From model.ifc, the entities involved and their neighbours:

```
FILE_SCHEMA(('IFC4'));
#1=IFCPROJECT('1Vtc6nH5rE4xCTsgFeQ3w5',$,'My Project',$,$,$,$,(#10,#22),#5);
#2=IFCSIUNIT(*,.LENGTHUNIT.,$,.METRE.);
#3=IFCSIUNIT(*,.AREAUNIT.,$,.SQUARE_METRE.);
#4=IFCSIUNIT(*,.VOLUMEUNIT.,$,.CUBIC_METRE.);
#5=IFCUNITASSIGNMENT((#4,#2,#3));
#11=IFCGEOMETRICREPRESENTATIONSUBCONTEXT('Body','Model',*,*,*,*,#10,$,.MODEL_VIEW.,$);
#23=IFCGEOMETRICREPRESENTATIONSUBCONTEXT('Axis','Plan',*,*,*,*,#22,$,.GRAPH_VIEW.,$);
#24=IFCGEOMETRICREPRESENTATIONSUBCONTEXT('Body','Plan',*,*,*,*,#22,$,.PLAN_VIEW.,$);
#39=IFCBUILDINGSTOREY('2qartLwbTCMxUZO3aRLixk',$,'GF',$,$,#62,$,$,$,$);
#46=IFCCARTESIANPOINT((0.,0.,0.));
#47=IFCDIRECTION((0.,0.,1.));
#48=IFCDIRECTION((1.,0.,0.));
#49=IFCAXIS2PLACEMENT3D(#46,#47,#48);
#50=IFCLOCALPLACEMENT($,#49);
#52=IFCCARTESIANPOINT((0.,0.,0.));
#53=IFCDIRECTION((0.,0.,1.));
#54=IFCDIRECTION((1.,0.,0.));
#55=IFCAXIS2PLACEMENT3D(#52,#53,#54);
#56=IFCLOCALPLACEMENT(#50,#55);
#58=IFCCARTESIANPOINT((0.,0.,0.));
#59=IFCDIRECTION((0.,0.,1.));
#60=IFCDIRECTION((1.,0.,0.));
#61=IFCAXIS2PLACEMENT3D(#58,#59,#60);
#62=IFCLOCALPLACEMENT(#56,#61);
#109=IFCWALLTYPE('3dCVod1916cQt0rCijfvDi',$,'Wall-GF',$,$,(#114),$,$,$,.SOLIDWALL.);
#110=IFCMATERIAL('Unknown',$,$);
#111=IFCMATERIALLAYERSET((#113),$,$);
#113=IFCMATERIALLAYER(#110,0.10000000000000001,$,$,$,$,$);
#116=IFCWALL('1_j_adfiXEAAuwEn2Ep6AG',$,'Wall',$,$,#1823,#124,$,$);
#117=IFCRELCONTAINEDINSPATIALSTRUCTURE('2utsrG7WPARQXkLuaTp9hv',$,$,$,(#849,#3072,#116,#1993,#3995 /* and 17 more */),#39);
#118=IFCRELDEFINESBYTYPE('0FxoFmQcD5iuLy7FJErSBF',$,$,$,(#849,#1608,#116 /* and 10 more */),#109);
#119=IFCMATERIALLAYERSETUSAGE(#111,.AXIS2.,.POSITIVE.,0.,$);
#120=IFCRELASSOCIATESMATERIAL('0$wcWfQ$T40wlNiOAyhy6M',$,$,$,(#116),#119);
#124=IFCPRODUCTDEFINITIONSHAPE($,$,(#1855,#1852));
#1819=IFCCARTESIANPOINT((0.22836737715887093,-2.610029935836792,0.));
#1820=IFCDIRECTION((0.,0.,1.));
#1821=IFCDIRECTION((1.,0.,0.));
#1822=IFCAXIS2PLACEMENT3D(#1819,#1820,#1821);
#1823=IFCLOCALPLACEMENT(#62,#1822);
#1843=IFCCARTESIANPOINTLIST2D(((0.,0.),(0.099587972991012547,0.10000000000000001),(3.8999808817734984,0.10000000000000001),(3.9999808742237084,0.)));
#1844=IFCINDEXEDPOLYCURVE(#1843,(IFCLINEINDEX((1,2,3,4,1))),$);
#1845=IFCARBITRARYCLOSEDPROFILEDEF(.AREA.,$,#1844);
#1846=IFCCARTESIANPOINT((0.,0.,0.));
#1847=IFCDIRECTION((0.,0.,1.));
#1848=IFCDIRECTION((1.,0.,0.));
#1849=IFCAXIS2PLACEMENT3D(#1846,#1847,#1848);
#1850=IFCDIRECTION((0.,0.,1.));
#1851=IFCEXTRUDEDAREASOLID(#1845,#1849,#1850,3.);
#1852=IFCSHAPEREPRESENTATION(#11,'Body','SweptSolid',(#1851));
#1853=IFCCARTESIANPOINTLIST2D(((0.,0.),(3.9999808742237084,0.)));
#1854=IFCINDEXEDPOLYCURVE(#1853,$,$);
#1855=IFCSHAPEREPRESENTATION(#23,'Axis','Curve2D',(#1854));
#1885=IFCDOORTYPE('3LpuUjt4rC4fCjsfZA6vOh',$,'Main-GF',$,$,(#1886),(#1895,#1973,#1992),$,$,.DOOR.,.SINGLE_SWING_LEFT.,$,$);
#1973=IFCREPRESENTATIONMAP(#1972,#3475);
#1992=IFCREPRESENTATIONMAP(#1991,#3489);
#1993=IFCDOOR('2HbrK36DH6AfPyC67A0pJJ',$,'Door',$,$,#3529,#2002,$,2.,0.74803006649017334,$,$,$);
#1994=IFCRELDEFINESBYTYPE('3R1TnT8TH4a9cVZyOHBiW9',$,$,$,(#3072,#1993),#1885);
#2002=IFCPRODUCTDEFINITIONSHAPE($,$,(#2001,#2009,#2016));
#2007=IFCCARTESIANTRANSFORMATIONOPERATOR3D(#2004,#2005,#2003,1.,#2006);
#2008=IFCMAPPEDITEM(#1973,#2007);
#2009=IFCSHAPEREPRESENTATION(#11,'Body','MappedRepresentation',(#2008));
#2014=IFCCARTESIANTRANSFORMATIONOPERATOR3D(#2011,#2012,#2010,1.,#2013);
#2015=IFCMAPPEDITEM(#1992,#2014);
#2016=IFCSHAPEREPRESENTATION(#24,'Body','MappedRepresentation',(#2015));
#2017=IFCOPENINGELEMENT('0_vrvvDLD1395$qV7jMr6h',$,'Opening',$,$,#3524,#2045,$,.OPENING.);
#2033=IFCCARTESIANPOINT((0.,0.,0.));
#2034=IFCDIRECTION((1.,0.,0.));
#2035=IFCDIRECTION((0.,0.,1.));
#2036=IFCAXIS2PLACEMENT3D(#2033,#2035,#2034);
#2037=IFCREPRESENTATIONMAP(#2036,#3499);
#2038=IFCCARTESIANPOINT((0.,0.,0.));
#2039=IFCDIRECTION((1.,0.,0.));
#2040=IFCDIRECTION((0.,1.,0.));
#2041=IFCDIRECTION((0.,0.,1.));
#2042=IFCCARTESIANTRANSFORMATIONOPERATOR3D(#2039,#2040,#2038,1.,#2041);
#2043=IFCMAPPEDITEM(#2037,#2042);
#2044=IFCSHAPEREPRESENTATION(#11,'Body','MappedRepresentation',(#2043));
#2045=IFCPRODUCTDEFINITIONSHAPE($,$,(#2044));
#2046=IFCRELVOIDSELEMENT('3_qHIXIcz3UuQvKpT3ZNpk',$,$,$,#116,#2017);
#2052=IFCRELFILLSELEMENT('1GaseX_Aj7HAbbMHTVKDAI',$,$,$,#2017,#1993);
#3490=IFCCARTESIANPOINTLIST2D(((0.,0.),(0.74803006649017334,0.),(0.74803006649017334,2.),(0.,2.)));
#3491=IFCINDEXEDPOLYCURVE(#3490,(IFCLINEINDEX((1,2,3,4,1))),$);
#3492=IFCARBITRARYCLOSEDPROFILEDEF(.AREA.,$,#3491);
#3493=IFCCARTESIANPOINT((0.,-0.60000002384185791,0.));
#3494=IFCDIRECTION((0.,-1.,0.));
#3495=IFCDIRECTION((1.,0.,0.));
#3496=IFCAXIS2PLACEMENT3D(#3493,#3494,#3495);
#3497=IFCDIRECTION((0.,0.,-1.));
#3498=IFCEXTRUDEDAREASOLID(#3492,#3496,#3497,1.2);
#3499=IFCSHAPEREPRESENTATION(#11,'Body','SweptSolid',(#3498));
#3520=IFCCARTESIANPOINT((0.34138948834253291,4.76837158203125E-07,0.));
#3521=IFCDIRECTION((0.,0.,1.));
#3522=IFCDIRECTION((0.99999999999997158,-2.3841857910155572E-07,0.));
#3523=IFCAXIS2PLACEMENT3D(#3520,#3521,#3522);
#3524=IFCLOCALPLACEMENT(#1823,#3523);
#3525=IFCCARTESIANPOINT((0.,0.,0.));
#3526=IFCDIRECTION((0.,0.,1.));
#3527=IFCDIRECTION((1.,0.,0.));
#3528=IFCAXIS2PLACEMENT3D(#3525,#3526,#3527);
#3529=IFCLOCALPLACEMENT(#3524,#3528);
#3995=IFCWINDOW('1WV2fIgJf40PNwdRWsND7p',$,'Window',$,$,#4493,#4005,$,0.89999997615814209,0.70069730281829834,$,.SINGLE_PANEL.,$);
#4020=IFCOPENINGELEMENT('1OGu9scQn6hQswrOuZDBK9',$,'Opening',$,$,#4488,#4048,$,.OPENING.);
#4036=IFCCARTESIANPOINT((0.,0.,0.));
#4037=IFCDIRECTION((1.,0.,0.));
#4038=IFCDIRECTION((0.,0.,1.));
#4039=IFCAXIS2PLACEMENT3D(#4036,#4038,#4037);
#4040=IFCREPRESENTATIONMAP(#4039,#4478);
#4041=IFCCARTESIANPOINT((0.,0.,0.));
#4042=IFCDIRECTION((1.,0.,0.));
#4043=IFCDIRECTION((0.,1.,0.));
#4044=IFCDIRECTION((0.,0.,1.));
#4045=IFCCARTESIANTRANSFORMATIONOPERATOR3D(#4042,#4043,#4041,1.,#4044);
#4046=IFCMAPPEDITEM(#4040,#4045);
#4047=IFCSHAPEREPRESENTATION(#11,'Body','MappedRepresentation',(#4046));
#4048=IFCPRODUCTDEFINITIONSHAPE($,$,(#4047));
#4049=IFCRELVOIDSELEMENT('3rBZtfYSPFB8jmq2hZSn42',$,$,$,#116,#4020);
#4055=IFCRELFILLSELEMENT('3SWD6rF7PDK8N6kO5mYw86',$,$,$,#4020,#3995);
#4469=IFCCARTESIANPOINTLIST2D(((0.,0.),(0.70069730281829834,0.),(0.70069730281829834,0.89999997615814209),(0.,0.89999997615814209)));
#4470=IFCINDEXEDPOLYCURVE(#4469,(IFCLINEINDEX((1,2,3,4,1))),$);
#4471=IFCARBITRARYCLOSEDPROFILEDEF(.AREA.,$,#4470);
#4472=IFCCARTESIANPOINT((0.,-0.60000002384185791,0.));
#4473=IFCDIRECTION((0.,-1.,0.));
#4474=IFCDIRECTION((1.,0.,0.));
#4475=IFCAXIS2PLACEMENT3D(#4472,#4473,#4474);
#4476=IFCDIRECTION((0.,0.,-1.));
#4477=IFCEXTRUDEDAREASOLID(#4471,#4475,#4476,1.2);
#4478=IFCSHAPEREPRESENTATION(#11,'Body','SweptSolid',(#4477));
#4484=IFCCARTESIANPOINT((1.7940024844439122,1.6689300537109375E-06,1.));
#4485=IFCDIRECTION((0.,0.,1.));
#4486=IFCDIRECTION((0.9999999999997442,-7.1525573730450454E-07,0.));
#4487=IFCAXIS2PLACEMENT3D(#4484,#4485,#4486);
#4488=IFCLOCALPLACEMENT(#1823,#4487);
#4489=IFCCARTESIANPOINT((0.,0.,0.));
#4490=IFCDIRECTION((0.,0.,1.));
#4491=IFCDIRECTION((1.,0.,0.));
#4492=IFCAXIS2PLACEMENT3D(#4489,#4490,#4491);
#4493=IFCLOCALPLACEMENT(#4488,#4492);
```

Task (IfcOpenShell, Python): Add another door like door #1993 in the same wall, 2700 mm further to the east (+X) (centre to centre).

```python
import ifcopenshell
import ifcopenshell.api.feature
import ifcopenshell.api.geometry
import ifcopenshell.api.root
import ifcopenshell.geom
import ifcopenshell.util.element
import ifcopenshell.util.placement
import ifcopenshell.util.shape
import ifcopenshell.util.unit

model = ifcopenshell.open("model.ifc")
unit_scale = ifcopenshell.util.unit.calculate_unit_scale(model)
settings = ifcopenshell.geom.settings()


def volume(element):
    """Net volume in cubic metres, openings subtracted."""
    shape = ifcopenshell.geom.create_shape(settings, element)
    return ifcopenshell.util.shape.get_volume(shape.geometry)


door = model.by_guid("2HbrK36DH6AfPyC67A0pJJ")
opening = door.FillsVoids[0].RelatingOpeningElement
wall = opening.VoidsElements[0].RelatingBuildingElement
before = volume(wall)
shift = ifcopenshell.util.placement.get_local_placement(wall.ObjectPlacement)[:3, 0] * 2.7 / unit_scale

# copy_class copies the void relationship, type, container and properties, but no geometry.
new_opening = ifcopenshell.api.root.copy_class(model, product=opening)
new_opening.Representation = ifcopenshell.util.element.copy_deep(
    model, opening.Representation, exclude=["IfcGeometricRepresentationContext", "IfcRepresentationMap"]
)
new_door = ifcopenshell.api.root.copy_class(model, product=door)
new_door.Representation = ifcopenshell.util.element.copy_deep(
    model, door.Representation, exclude=["IfcGeometricRepresentationContext", "IfcRepresentationMap"]
)
ifcopenshell.api.feature.add_filling(model, opening=new_opening, element=new_door)

for old, new in ((opening, new_opening), (door, new_door)):
    matrix = ifcopenshell.util.placement.get_local_placement(old.ObjectPlacement)
    matrix[:3, 3] += shift
    ifcopenshell.api.geometry.edit_object_placement(model, product=new, matrix=matrix, is_si=False)

after = volume(wall)

print(f"wall volume {before:.3f} -> {after:.3f} m3")

model.write("model-out.ifc")
```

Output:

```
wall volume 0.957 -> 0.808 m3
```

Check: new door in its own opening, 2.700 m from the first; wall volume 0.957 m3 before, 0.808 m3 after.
